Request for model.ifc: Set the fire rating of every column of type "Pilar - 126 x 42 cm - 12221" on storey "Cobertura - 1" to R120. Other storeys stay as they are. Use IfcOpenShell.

First a look at what the model holds.

```python
import ifcopenshell
import ifcopenshell.util.element

model = ifcopenshell.open("model.ifc")
print(model.schema)
storey = next(s for s in model.by_type("IfcBuildingStorey") if s.Name == "Cobertura - 1")
columns = [e for e in ifcopenshell.util.element.get_decomposition(storey) if e.is_a("IfcColumn")]
seen = {}
for e in columns:
    element_type = ifcopenshell.util.element.get_type(e)
    key = (element_type.Name if element_type != e and element_type else None, ifcopenshell.util.element.get_pset(e, "Pset_ColumnCommon", "FireRating"))
    seen[key] = seen.get(key, 0) + 1
for (name, value), count in sorted(seen.items(), key=str):
    print(count, "x", name, "|", value)
```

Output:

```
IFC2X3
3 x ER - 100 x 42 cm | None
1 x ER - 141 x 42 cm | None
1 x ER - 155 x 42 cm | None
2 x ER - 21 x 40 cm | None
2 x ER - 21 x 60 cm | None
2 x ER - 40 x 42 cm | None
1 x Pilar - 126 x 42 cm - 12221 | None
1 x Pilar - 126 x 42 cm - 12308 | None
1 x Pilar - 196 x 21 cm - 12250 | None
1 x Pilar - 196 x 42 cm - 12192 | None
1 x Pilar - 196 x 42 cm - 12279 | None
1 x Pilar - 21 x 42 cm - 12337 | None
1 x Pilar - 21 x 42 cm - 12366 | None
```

```python
import ifcopenshell
import ifcopenshell.api.pset
import ifcopenshell.util.element

model = ifcopenshell.open("model.ifc")

storey = next(s for s in model.by_type("IfcBuildingStorey") if s.Name == "Cobertura - 1")
columns = [e for e in ifcopenshell.util.element.get_decomposition(storey) if e.is_a("IfcColumn")]

count = 0
for e in columns:
    element_type = ifcopenshell.util.element.get_type(e)
    if element_type in (None, e) or element_type.Name != "Pilar - 126 x 42 cm - 12221":
        continue
    # add_pset returns the element's existing set when there is one.
    pset = ifcopenshell.api.pset.add_pset(model, product=e, name="Pset_ColumnCommon")
    ifcopenshell.api.pset.edit_pset(model, pset=pset, properties={"FireRating": "R120"})
    count += 1

print(count, "columns updated")

model.write("model_updated.ifc")
```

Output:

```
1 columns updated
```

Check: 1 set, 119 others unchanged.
